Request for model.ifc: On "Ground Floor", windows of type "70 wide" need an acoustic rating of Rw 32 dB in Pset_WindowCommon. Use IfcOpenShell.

First a look at what the model holds.

```python
import ifcopenshell
import ifcopenshell.util.element

model = ifcopenshell.open("model.ifc")
print(model.schema)
storey = next(s for s in model.by_type("IfcBuildingStorey") if s.Name == "Ground Floor")
windows = [e for e in ifcopenshell.util.element.get_decomposition(storey) if e.is_a("IfcWindow")]
seen = {}
for e in windows:
    element_type = ifcopenshell.util.element.get_type(e)
    key = (element_type.Name if element_type != e and element_type else None, ifcopenshell.util.element.get_pset(e, "Pset_WindowCommon", "AcousticRating"))
    seen[key] = seen.get(key, 0) + 1
for (name, value), count in sorted(seen.items(), key=str):
    print(count, "x", name, "|", value)
```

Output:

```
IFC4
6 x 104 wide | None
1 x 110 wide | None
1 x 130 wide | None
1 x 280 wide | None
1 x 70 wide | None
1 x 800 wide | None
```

```python
import ifcopenshell
import ifcopenshell.api.pset
import ifcopenshell.util.element

model = ifcopenshell.open("model.ifc")

storey = next(s for s in model.by_type("IfcBuildingStorey") if s.Name == "Ground Floor")
windows = [e for e in ifcopenshell.util.element.get_decomposition(storey) if e.is_a("IfcWindow")]

count = 0
for e in windows:
    element_type = ifcopenshell.util.element.get_type(e)
    if element_type in (None, e) or element_type.Name != "70 wide":
        continue
    # add_pset returns the element's existing set when there is one.
    pset = ifcopenshell.api.pset.add_pset(model, product=e, name="Pset_WindowCommon")
    ifcopenshell.api.pset.edit_pset(model, pset=pset, properties={"AcousticRating": "Rw 32 dB"})
    count += 1

print(count, "windows updated")

model.write("model_rev.ifc")
```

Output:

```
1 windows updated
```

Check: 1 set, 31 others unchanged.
